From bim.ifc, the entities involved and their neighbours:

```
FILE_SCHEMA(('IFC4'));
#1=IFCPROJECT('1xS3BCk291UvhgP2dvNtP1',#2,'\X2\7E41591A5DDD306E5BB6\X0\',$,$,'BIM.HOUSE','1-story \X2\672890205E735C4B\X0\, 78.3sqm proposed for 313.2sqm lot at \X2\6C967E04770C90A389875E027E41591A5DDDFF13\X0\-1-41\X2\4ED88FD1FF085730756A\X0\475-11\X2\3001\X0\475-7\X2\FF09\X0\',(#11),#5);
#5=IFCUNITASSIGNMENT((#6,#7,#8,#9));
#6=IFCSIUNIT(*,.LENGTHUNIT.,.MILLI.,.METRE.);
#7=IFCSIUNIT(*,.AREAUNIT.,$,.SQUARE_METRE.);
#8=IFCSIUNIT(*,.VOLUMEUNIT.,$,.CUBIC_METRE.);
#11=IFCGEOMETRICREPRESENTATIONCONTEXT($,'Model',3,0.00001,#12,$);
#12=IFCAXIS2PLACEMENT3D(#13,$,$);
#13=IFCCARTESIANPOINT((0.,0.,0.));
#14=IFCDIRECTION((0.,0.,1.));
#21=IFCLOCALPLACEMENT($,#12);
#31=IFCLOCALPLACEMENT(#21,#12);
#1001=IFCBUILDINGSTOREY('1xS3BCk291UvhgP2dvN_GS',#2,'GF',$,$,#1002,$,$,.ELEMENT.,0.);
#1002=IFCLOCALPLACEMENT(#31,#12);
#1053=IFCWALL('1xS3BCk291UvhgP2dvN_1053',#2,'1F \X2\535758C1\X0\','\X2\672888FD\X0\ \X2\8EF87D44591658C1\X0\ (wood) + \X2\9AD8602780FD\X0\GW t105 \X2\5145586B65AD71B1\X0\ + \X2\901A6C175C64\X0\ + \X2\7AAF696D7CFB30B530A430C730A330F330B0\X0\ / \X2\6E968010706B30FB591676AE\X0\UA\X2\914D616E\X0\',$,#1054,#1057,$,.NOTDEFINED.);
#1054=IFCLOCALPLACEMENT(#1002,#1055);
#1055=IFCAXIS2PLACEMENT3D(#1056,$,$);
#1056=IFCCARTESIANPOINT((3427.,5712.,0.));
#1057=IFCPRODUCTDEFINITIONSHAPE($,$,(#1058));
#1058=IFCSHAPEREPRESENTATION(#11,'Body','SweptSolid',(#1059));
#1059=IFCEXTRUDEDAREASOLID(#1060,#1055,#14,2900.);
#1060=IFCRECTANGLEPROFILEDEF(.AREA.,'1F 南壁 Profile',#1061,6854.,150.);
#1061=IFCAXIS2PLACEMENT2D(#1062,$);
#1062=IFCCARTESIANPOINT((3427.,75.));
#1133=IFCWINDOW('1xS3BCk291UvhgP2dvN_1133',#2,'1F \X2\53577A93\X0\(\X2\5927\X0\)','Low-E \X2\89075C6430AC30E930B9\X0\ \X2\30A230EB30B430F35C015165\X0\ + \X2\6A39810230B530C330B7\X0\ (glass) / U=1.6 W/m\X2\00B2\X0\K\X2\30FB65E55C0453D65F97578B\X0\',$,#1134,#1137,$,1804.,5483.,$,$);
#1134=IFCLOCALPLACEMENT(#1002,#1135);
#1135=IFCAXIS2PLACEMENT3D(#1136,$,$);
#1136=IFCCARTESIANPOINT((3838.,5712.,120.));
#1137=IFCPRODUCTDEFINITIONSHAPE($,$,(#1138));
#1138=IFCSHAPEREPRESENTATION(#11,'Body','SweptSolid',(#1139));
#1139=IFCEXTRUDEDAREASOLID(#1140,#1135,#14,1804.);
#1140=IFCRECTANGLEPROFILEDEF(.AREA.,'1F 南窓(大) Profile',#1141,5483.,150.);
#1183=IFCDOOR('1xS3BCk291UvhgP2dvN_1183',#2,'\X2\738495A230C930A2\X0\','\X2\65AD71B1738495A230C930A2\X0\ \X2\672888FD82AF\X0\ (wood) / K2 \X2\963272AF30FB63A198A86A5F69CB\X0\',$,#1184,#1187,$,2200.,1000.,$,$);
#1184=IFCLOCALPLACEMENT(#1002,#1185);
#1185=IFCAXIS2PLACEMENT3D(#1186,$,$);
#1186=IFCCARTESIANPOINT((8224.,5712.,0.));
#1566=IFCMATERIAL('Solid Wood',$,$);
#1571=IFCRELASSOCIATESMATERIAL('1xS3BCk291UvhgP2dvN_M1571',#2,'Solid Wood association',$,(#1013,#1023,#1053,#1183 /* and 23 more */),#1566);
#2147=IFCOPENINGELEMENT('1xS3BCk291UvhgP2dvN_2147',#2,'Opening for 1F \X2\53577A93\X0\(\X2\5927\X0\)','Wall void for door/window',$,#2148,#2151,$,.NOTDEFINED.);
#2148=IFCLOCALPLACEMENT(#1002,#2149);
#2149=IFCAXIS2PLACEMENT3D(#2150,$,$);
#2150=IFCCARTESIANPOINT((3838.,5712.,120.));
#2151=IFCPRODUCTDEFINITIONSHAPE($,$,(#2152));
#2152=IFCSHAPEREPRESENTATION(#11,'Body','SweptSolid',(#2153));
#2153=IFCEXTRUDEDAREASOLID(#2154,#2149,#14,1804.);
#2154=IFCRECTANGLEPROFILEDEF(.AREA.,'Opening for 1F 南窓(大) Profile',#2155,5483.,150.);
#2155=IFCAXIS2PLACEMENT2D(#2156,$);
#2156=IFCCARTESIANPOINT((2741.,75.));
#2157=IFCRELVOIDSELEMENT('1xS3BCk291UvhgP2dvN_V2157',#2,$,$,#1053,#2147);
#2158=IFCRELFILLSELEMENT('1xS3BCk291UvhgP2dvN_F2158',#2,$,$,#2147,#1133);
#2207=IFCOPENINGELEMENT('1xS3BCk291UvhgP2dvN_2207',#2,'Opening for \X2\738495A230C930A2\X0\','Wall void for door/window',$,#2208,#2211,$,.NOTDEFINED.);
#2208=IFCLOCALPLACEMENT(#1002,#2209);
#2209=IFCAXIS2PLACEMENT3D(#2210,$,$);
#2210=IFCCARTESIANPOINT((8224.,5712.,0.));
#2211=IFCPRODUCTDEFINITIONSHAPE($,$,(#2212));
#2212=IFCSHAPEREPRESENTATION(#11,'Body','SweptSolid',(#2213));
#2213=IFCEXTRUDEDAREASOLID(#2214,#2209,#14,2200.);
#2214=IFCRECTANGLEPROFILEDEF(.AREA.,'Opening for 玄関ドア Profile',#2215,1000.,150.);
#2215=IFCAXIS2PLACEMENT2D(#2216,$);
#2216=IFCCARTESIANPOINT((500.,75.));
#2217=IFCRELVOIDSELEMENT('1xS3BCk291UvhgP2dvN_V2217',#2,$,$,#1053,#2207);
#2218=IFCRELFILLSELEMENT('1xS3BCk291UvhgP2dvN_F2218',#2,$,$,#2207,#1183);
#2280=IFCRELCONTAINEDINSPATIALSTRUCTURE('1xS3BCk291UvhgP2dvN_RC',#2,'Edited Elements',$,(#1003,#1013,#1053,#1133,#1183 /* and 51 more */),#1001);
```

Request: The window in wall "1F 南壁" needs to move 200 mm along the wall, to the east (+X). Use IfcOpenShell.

```python
import ifcopenshell
import ifcopenshell.api.geometry
import ifcopenshell.util.placement

model = ifcopenshell.open("bim.ifc")

window = model.by_guid("1xS3BCk291UvhgP2dvN_1133")
opening = window.FillsVoids[0].RelatingOpeningElement
wall = opening.VoidsElements[0].RelatingBuildingElement

wall_matrix = ifcopenshell.util.placement.get_local_placement(wall.ObjectPlacement)
shift = wall_matrix[:3, 0] * 200.0
before = ifcopenshell.util.placement.get_local_placement(window.ObjectPlacement)[:3, 3].copy()

# The window is not placed relative to its opening, so move both.
for product in (opening, window):
    matrix = ifcopenshell.util.placement.get_local_placement(product.ObjectPlacement)
    matrix[:3, 3] += shift
    ifcopenshell.api.geometry.edit_object_placement(model, product=product, matrix=matrix, is_si=False)

after = ifcopenshell.util.placement.get_local_placement(window.ObjectPlacement)[:3, 3]
print("window moved by", (after - before).round(3) + 0.0)

model.write("bim_updated.ifc")
```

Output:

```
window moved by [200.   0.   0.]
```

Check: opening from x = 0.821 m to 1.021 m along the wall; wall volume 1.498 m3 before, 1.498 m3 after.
